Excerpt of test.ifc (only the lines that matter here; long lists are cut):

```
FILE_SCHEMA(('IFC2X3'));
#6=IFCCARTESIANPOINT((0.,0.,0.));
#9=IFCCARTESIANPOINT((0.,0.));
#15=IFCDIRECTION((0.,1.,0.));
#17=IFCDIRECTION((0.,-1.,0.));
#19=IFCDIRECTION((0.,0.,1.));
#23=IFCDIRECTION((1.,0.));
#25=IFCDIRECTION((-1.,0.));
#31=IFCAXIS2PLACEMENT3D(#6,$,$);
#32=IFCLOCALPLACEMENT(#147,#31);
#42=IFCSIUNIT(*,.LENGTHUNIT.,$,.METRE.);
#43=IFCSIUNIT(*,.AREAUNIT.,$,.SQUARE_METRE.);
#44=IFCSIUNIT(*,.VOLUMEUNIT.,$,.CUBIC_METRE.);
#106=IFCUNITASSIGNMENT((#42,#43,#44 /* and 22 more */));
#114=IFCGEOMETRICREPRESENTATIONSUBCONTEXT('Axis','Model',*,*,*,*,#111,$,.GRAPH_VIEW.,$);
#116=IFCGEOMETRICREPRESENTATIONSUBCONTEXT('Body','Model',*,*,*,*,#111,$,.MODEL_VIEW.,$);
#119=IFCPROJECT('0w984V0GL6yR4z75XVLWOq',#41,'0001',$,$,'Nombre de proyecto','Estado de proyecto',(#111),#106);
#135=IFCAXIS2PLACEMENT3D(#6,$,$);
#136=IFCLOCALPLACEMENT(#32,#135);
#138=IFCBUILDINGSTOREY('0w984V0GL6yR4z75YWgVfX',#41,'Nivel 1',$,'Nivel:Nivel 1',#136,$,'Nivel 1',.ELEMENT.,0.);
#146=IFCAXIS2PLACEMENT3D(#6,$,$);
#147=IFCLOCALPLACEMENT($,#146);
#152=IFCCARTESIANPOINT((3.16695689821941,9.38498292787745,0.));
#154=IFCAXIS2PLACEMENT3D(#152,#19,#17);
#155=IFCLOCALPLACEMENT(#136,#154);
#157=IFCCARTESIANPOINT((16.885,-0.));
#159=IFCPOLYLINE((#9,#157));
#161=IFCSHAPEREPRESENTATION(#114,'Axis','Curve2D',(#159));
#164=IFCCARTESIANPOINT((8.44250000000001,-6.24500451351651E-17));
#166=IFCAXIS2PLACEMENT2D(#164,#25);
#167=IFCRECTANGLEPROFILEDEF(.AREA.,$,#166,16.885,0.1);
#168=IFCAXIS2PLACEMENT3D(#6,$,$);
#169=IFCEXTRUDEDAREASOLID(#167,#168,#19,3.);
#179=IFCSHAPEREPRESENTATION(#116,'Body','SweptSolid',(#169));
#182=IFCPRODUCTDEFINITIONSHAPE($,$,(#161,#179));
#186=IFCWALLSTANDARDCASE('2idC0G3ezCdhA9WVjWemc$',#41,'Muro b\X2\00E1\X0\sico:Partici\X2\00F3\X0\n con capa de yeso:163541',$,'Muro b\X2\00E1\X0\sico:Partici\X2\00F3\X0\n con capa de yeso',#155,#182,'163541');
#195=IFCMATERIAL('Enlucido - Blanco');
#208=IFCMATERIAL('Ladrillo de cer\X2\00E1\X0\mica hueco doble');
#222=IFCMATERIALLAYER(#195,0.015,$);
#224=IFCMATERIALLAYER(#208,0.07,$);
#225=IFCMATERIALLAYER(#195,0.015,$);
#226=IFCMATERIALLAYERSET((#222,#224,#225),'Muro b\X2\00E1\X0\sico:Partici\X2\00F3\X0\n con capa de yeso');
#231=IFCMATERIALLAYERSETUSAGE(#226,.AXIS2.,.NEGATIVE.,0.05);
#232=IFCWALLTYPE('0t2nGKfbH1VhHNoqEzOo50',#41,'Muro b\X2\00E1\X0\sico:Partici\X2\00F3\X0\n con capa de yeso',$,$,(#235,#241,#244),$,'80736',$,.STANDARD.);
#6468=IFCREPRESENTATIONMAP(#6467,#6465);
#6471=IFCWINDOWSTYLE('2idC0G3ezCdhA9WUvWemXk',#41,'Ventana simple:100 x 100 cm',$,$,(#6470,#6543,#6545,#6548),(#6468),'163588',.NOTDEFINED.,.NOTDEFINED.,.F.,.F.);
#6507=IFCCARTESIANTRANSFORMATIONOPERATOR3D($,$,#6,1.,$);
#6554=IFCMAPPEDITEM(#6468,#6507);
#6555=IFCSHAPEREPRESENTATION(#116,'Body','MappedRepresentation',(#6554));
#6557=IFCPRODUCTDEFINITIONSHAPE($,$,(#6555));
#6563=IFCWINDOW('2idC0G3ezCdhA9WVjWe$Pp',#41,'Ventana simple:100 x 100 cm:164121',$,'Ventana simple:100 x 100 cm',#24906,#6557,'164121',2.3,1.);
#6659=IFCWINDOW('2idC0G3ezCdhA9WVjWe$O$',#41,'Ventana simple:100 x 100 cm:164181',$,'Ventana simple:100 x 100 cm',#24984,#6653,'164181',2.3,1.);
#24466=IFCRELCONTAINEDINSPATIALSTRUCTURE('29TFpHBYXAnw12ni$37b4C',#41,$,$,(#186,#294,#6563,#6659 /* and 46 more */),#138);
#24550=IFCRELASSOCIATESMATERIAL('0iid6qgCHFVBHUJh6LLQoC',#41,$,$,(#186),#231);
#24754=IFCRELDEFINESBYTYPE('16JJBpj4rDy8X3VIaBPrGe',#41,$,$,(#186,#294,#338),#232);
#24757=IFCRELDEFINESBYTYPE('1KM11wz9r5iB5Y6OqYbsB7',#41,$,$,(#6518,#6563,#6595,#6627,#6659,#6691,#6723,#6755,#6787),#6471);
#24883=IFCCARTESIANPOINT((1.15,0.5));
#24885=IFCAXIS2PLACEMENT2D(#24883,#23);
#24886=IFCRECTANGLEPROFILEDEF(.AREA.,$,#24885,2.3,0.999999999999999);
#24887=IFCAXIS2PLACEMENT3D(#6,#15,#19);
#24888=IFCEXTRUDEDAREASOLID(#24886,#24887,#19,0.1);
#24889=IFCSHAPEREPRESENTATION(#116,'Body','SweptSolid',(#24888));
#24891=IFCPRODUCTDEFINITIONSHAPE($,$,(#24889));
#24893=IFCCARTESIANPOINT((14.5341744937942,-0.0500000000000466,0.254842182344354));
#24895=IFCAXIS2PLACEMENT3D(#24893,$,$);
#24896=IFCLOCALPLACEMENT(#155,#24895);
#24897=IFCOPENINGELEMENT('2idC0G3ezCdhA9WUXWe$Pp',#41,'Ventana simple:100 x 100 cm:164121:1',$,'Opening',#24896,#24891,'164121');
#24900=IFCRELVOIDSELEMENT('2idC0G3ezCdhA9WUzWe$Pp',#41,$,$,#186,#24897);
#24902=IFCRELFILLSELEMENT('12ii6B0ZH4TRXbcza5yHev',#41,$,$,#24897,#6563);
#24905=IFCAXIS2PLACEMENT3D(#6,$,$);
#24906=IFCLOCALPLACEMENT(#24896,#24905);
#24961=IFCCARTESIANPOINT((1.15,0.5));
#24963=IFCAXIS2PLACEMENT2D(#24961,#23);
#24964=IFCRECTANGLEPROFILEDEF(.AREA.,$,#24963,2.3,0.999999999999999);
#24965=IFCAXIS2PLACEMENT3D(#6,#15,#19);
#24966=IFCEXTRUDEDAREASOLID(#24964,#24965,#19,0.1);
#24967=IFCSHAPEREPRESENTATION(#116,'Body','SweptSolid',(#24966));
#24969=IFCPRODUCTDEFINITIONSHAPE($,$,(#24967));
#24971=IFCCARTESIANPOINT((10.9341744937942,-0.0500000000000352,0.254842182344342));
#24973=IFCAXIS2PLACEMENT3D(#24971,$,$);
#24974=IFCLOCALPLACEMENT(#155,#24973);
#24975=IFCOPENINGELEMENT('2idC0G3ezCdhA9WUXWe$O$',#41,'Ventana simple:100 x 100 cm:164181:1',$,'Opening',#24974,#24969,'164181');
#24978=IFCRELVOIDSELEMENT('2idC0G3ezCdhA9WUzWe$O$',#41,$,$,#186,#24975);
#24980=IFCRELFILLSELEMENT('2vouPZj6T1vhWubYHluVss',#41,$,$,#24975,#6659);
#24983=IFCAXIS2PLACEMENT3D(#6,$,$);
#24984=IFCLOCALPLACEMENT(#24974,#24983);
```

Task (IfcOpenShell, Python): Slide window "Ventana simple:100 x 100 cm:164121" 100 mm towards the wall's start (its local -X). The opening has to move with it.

```python
import ifcopenshell
import ifcopenshell.api.geometry
import ifcopenshell.util.placement

model = ifcopenshell.open("test.ifc")

window = model.by_guid("2idC0G3ezCdhA9WVjWe$Pp")
opening = window.FillsVoids[0].RelatingOpeningElement
wall = opening.VoidsElements[0].RelatingBuildingElement

wall_matrix = ifcopenshell.util.placement.get_local_placement(wall.ObjectPlacement)
shift = wall_matrix[:3, 0] * -0.1
before = ifcopenshell.util.placement.get_local_placement(window.ObjectPlacement)[:3, 3].copy()

# The window is placed relative to its opening, so it follows when the opening moves.
matrix = ifcopenshell.util.placement.get_local_placement(opening.ObjectPlacement)
matrix[:3, 3] += shift
ifcopenshell.api.geometry.edit_object_placement(
    model, product=opening, matrix=matrix, is_si=False, should_transform_children=True
)

after = ifcopenshell.util.placement.get_local_placement(window.ObjectPlacement)[:3, 3]
print("window moved by", (after - before).round(3) + 0.0)

model.write("test_updated.ifc")
```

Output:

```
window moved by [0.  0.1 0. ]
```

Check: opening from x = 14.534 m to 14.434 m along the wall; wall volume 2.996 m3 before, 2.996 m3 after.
